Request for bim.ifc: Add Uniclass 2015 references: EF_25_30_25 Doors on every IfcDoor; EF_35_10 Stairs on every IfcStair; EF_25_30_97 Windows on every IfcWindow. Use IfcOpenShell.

First a look at what the model holds.

```python
import ifcopenshell

model = ifcopenshell.open("bim.ifc")
print(model.schema)
print("classifications:", [c.Name for c in model.by_type("IfcClassification")])
for ifc_class in ("IfcDoor", "IfcRoof", "IfcStair", "IfcWall", "IfcWindow"):
    print(ifc_class, len(model.by_type(ifc_class)))
```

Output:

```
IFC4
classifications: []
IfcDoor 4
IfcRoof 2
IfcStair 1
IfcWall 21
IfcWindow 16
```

```python
import ifcopenshell
import ifcopenshell.api.classification

model = ifcopenshell.open("bim.ifc")

system = ifcopenshell.api.classification.add_classification(model, classification="Uniclass 2015")

codes = {
    "IfcDoor": ("EF_25_30_25", "Doors"),
    "IfcStair": ("EF_35_10", "Stairs"),
    "IfcWindow": ("EF_25_30_97", "Windows"),
}
for ifc_class, (code, name) in codes.items():
    products = model.by_type(ifc_class)
    ifcopenshell.api.classification.add_reference(
        model, products=products, classification=system, identification=code, name=name
    )
    print(code, len(products))

model.write("bim_rev.ifc")
```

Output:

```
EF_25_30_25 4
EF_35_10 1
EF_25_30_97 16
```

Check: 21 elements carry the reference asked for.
